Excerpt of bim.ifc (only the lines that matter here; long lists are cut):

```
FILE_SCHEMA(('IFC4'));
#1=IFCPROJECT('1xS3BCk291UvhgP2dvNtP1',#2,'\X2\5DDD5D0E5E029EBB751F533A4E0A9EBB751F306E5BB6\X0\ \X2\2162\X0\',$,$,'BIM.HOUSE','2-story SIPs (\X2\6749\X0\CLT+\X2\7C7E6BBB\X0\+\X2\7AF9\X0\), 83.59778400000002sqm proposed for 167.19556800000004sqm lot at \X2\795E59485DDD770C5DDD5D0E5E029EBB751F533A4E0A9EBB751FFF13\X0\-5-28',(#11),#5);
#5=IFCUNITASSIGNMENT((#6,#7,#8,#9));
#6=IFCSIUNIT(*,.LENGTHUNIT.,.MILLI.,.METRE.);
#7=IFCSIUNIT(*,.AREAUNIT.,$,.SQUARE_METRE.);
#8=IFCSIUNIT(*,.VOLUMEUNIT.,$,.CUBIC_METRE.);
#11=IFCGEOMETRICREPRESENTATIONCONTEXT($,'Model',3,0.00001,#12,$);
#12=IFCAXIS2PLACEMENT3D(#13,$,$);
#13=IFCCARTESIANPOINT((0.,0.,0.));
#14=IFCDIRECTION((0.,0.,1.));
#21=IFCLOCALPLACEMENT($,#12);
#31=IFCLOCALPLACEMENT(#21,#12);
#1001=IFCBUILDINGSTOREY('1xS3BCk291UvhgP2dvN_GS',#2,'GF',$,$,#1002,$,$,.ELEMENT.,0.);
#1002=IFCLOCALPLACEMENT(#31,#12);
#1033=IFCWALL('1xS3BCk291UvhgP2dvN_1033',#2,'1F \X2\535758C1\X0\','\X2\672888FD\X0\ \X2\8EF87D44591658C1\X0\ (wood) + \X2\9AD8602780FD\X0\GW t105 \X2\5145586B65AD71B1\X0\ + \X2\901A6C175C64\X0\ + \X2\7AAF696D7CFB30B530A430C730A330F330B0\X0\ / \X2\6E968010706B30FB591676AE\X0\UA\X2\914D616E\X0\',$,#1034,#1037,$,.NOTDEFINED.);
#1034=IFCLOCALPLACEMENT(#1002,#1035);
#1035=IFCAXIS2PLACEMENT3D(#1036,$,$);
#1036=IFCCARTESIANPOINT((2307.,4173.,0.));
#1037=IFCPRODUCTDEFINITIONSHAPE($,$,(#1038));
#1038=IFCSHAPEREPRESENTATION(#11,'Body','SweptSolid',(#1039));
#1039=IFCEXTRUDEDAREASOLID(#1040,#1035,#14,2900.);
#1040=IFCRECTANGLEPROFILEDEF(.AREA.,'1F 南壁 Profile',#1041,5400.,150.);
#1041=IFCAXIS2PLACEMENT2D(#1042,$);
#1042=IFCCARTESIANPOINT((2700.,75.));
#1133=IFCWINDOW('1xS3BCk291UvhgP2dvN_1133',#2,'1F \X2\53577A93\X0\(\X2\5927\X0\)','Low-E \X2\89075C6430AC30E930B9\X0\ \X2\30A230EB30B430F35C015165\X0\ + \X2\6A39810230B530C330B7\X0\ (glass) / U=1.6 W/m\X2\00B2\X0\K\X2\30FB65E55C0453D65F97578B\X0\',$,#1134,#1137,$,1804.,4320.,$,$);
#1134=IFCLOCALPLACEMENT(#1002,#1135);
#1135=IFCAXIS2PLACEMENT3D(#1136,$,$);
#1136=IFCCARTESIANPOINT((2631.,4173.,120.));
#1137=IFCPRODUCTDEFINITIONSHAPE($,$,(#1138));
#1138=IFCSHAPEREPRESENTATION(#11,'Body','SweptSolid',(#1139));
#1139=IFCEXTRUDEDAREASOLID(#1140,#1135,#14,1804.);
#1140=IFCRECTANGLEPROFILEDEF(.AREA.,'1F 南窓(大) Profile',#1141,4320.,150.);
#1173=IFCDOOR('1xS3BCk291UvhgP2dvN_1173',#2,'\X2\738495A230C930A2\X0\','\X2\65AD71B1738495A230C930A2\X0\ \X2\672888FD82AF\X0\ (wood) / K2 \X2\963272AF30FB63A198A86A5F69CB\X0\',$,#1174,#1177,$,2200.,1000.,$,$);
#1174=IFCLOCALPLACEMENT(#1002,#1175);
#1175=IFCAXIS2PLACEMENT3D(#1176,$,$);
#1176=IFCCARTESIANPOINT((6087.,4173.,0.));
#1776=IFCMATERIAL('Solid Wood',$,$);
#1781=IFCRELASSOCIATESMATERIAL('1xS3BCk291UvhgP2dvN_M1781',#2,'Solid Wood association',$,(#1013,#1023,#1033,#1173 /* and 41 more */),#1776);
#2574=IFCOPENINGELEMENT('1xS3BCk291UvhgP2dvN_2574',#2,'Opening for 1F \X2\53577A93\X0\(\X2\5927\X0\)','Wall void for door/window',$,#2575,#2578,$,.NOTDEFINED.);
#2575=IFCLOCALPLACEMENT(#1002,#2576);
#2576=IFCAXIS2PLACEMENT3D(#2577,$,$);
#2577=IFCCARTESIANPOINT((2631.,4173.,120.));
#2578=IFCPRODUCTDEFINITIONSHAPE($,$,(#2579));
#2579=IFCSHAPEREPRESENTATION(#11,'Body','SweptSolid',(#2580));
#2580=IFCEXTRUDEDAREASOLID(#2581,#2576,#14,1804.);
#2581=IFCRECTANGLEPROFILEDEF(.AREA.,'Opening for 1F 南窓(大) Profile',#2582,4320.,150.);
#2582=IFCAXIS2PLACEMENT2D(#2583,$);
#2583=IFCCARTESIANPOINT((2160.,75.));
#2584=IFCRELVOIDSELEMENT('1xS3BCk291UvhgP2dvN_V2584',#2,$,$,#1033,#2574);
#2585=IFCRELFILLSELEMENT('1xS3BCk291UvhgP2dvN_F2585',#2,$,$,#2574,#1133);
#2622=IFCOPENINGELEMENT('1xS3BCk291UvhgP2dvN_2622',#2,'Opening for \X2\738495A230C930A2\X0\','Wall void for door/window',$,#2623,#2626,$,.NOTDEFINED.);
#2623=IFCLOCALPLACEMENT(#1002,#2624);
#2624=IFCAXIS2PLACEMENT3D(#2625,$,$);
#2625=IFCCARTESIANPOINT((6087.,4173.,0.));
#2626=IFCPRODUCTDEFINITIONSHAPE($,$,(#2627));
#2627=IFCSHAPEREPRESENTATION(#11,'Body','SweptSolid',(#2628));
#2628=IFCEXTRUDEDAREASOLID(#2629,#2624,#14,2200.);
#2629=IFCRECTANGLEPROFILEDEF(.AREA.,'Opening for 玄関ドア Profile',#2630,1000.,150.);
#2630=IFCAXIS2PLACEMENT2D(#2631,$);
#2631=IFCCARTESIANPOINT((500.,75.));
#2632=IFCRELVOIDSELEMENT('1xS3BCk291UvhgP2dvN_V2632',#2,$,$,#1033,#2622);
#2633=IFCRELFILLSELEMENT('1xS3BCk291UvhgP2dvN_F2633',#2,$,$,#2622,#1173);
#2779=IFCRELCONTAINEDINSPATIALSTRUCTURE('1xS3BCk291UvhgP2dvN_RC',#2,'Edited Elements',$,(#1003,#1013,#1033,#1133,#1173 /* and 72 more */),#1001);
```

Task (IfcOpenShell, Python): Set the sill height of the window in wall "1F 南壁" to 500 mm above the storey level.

```python
import numpy as np
import ifcopenshell
import ifcopenshell.api.geometry
import ifcopenshell.geom
import ifcopenshell.util.element
import ifcopenshell.util.placement
import ifcopenshell.util.shape
import ifcopenshell.util.unit

model = ifcopenshell.open("bim.ifc")
unit_scale = ifcopenshell.util.unit.calculate_unit_scale(model)

window = model.by_guid("1xS3BCk291UvhgP2dvN_1133")
opening = window.FillsVoids[0].RelatingOpeningElement
storey = ifcopenshell.util.element.get_container(window, ifc_class="IfcBuildingStorey")
level = ifcopenshell.util.placement.get_local_placement(storey.ObjectPlacement)[2, 3]

# The opening's origin need not be at the sill, so measure its lowest point.
shape = ifcopenshell.geom.create_shape(ifcopenshell.geom.settings(), opening)
bottom = ifcopenshell.util.shape.get_shape_bottom_elevation(shape, shape.geometry) / unit_scale
dz = level + 500.0 - bottom

shift = np.array([0.0, 0.0, dz])
# The window is not placed relative to its opening, so move both.
for product in (opening, window):
    matrix = ifcopenshell.util.placement.get_local_placement(product.ObjectPlacement)
    matrix[:3, 3] += shift
    ifcopenshell.api.geometry.edit_object_placement(model, product=product, matrix=matrix, is_si=False)

print(f"moved by {dz * unit_scale:+.3f} m")

model.write("bim-out.ifc")
```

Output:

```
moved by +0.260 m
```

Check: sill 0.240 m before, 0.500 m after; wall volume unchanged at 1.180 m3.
